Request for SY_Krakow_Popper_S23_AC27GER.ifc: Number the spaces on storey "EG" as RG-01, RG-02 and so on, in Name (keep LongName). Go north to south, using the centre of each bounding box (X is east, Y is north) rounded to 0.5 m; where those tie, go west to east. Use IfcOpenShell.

First a look at what the model holds.

```python
import ifcopenshell
import ifcopenshell.util.element
import ifcopenshell.util.placement

model = ifcopenshell.open("SY_Krakow_Popper_S23_AC27GER.ifc")
print(model.schema)
storey = next(s for s in model.by_type("IfcBuildingStorey") if s.Name == "EG")
spaces = [e for e in ifcopenshell.util.element.get_decomposition(storey) if e.is_a("IfcSpace")]
for e in sorted(spaces, key=lambda e: e.id()):
    origin = ifcopenshell.util.placement.get_local_placement(e.ObjectPlacement)[:3, 3]
    print(e.id(), e.Name, e.LongName, origin.round(2) + 0.0, sep=" | ")
```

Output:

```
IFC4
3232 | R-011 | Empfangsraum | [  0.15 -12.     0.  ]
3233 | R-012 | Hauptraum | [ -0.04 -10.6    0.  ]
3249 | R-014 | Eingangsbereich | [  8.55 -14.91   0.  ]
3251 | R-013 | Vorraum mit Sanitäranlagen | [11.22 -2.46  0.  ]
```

```python
import ifcopenshell
import ifcopenshell.geom
import ifcopenshell.util.element
import ifcopenshell.util.shape

model = ifcopenshell.open("SY_Krakow_Popper_S23_AC27GER.ifc")
settings = ifcopenshell.geom.settings()
settings.set("use-world-coords", True)


def centre(element):
    shape = ifcopenshell.geom.create_shape(settings, element)
    return ifcopenshell.util.shape.get_bbox_centroid(shape.geometry)


storey = next(s for s in model.by_type("IfcBuildingStorey") if s.Name == "EG")
spaces = [e for e in ifcopenshell.util.element.get_decomposition(storey) if e.is_a("IfcSpace")]

# Insertion points can sit at a corner or the storey origin, so sort by the geometry (in metres).
centres = {e: centre(e) for e in spaces}
spaces.sort(key=lambda e: (-round(centres[e][1] / 0.5), centres[e][0]))

for i, e in enumerate(spaces, start=1):
    number = f"RG-{i:02d}"
    e.Name = number
    print(e.id(), number)

model.write("SY_Krakow_Popper_S23_AC27GER_updated.ifc")
```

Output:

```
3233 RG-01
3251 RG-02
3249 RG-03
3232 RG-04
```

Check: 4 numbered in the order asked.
